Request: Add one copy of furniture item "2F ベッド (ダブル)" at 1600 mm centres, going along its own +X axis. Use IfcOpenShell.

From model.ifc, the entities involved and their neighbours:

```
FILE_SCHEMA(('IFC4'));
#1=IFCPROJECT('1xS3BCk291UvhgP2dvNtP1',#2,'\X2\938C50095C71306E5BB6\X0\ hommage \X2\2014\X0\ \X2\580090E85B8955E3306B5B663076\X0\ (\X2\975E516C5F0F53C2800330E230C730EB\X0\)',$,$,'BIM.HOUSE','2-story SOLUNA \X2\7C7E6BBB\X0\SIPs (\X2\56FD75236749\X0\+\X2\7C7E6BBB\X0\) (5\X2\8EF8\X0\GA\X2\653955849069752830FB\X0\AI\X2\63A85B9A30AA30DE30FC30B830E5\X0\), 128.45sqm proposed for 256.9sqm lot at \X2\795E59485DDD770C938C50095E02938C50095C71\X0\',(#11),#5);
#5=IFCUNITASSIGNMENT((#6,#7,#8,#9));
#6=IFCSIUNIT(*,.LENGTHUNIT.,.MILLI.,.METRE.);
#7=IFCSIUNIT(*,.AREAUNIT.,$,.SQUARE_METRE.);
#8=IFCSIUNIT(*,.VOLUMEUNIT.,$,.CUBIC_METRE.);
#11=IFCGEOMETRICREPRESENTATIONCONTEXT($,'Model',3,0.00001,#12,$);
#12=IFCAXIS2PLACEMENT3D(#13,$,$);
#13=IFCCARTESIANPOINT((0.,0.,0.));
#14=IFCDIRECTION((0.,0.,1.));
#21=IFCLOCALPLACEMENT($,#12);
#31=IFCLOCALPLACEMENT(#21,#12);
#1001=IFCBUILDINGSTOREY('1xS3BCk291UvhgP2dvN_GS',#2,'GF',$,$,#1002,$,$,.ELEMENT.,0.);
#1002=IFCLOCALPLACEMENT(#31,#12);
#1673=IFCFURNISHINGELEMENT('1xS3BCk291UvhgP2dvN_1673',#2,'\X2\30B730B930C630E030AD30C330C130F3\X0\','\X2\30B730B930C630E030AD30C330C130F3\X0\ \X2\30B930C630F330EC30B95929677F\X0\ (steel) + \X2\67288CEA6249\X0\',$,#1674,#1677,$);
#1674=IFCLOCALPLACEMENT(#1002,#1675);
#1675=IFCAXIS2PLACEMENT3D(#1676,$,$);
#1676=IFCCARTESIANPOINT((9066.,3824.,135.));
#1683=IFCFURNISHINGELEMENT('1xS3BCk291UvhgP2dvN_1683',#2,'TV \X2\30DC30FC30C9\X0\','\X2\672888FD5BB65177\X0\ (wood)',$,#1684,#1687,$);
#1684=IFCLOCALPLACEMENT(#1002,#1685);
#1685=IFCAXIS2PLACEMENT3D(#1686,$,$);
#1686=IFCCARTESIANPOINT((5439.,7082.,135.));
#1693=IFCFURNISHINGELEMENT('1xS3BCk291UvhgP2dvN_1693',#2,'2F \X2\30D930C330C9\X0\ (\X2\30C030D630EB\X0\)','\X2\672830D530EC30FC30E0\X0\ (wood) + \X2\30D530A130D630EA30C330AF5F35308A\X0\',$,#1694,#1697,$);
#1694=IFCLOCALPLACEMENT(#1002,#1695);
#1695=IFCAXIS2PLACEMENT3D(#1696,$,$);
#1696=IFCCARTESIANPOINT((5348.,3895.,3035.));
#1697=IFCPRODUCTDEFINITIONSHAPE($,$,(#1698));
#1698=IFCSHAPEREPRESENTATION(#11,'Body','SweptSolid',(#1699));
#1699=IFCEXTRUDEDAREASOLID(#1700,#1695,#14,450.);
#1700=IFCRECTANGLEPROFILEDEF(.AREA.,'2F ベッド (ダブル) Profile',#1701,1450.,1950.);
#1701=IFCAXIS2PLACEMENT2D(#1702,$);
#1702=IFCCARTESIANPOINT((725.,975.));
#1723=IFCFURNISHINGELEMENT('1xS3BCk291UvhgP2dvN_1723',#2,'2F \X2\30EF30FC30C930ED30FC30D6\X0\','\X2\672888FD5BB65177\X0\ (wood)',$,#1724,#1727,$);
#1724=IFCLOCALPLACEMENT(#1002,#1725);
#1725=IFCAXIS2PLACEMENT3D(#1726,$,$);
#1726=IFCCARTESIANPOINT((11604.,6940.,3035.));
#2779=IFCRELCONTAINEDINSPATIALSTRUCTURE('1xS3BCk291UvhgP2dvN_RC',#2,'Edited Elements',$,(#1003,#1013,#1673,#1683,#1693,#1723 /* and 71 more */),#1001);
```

```python
import ifcopenshell
import ifcopenshell.api.geometry
import ifcopenshell.api.root
import ifcopenshell.util.element
import ifcopenshell.util.placement
import ifcopenshell.util.unit

model = ifcopenshell.open("model.ifc")
unit_scale = ifcopenshell.util.unit.calculate_unit_scale(model)


def reuse_history(source, copy):
    """copy_class also copies each property set's owner history, people and application; keep the originals."""
    for rel in copy.IsDefinedBy:
        if rel.is_a("IfcRelDefinesByProperties") and (history := rel.RelatingPropertyDefinition.OwnerHistory):
            rel.RelatingPropertyDefinition.OwnerHistory = source.OwnerHistory
            ifcopenshell.util.element.remove_deep2(model, history)


source = model.by_guid("1xS3BCk291UvhgP2dvN_1693")
base = ifcopenshell.util.placement.get_local_placement(source.ObjectPlacement)
step = base[:3, 0] * 1.6 / unit_scale

for i in range(1, 2):
    copy = ifcopenshell.api.root.copy_class(model, product=source)
    copy.Representation = ifcopenshell.util.element.copy_deep(
        model, source.Representation, exclude=["IfcGeometricRepresentationContext", "IfcRepresentationMap"]
    )
    reuse_history(source, copy)
    matrix = base.copy()
    matrix[:3, 3] += i * step
    print("added at", matrix[:3, 3].round(3) + 0.0)
    ifcopenshell.api.geometry.edit_object_placement(model, product=copy, matrix=matrix, is_si=False)

model.write("model_updated.ifc")
```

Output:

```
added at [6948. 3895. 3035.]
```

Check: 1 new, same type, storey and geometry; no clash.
